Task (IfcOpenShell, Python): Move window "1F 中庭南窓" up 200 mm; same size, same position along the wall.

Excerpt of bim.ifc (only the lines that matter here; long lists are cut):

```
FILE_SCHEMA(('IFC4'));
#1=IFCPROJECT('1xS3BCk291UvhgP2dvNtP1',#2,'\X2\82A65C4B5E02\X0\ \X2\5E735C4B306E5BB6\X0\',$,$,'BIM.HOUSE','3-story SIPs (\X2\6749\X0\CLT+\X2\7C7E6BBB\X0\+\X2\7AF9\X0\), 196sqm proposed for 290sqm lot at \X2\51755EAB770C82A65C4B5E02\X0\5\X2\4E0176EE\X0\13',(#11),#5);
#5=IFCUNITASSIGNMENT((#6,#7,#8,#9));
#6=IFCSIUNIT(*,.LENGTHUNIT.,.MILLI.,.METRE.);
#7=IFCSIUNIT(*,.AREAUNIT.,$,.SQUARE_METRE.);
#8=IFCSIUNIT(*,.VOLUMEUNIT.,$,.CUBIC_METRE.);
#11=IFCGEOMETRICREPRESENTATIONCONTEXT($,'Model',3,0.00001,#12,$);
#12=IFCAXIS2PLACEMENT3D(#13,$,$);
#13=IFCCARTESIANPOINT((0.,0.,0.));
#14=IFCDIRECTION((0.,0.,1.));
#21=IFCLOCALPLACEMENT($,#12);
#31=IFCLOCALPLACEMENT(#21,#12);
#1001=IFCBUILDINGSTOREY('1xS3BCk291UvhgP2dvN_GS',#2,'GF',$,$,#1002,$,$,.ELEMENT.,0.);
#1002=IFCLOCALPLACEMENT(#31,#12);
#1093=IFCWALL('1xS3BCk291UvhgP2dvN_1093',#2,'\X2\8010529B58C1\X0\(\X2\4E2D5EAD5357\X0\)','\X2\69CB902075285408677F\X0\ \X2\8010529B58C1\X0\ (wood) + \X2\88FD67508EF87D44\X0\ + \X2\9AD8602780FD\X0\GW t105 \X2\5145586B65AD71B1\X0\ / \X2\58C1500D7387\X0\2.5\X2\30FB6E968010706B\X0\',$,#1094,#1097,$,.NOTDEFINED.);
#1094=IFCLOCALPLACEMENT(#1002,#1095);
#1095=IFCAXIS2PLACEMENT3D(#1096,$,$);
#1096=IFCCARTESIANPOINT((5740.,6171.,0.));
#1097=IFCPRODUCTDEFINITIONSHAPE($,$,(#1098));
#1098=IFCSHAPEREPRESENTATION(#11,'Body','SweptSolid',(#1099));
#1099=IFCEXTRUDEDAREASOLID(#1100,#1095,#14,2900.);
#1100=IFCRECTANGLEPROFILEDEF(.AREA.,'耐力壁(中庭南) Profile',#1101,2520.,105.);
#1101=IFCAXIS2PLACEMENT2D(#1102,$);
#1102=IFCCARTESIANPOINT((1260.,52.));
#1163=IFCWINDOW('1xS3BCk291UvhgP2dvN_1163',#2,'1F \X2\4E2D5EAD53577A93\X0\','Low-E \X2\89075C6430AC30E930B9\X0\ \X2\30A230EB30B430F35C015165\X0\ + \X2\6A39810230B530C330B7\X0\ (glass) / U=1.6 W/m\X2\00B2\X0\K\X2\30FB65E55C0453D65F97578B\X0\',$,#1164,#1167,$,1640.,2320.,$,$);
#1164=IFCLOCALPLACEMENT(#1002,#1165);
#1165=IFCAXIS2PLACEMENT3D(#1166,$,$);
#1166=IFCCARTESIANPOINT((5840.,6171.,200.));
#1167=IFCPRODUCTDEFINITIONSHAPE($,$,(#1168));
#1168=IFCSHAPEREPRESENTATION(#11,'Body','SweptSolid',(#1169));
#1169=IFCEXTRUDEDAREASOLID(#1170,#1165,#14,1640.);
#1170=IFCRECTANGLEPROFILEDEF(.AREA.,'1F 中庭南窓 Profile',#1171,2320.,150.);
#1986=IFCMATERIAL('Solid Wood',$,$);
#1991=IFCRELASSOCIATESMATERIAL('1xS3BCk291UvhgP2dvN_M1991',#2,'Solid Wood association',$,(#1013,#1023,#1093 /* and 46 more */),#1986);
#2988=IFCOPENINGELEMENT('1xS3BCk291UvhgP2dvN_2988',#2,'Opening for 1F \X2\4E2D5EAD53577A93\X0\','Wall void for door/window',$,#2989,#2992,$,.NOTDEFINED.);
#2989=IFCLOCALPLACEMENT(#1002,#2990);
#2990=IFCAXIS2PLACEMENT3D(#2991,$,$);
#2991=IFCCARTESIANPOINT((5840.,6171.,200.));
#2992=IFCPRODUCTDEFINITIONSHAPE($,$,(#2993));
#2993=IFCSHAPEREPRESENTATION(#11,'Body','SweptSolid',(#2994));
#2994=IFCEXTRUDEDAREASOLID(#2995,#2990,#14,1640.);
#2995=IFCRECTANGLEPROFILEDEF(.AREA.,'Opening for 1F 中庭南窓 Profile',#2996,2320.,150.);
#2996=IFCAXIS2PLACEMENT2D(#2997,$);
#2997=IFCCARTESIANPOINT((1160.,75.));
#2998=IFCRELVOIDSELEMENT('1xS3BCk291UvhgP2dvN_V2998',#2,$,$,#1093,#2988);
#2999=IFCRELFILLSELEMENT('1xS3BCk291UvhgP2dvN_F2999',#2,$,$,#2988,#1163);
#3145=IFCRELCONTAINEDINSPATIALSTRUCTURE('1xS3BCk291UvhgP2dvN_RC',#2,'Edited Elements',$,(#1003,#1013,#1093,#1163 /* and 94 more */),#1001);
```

```python
import numpy as np
import ifcopenshell
import ifcopenshell.api.geometry
import ifcopenshell.util.placement
import ifcopenshell.util.unit

model = ifcopenshell.open("bim.ifc")
unit_scale = ifcopenshell.util.unit.calculate_unit_scale(model)

window = model.by_id(1163)
opening = window.FillsVoids[0].RelatingOpeningElement
dz = 0.2 / unit_scale

shift = np.array([0.0, 0.0, dz])
# The window is not placed relative to its opening, so move both.
for product in (opening, window):
    matrix = ifcopenshell.util.placement.get_local_placement(product.ObjectPlacement)
    matrix[:3, 3] += shift
    ifcopenshell.api.geometry.edit_object_placement(model, product=product, matrix=matrix, is_si=False)

print(f"moved by {dz * unit_scale:+.3f} m")

model.write("bim_edited.ifc")
```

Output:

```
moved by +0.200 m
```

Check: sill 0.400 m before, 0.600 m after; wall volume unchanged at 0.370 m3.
